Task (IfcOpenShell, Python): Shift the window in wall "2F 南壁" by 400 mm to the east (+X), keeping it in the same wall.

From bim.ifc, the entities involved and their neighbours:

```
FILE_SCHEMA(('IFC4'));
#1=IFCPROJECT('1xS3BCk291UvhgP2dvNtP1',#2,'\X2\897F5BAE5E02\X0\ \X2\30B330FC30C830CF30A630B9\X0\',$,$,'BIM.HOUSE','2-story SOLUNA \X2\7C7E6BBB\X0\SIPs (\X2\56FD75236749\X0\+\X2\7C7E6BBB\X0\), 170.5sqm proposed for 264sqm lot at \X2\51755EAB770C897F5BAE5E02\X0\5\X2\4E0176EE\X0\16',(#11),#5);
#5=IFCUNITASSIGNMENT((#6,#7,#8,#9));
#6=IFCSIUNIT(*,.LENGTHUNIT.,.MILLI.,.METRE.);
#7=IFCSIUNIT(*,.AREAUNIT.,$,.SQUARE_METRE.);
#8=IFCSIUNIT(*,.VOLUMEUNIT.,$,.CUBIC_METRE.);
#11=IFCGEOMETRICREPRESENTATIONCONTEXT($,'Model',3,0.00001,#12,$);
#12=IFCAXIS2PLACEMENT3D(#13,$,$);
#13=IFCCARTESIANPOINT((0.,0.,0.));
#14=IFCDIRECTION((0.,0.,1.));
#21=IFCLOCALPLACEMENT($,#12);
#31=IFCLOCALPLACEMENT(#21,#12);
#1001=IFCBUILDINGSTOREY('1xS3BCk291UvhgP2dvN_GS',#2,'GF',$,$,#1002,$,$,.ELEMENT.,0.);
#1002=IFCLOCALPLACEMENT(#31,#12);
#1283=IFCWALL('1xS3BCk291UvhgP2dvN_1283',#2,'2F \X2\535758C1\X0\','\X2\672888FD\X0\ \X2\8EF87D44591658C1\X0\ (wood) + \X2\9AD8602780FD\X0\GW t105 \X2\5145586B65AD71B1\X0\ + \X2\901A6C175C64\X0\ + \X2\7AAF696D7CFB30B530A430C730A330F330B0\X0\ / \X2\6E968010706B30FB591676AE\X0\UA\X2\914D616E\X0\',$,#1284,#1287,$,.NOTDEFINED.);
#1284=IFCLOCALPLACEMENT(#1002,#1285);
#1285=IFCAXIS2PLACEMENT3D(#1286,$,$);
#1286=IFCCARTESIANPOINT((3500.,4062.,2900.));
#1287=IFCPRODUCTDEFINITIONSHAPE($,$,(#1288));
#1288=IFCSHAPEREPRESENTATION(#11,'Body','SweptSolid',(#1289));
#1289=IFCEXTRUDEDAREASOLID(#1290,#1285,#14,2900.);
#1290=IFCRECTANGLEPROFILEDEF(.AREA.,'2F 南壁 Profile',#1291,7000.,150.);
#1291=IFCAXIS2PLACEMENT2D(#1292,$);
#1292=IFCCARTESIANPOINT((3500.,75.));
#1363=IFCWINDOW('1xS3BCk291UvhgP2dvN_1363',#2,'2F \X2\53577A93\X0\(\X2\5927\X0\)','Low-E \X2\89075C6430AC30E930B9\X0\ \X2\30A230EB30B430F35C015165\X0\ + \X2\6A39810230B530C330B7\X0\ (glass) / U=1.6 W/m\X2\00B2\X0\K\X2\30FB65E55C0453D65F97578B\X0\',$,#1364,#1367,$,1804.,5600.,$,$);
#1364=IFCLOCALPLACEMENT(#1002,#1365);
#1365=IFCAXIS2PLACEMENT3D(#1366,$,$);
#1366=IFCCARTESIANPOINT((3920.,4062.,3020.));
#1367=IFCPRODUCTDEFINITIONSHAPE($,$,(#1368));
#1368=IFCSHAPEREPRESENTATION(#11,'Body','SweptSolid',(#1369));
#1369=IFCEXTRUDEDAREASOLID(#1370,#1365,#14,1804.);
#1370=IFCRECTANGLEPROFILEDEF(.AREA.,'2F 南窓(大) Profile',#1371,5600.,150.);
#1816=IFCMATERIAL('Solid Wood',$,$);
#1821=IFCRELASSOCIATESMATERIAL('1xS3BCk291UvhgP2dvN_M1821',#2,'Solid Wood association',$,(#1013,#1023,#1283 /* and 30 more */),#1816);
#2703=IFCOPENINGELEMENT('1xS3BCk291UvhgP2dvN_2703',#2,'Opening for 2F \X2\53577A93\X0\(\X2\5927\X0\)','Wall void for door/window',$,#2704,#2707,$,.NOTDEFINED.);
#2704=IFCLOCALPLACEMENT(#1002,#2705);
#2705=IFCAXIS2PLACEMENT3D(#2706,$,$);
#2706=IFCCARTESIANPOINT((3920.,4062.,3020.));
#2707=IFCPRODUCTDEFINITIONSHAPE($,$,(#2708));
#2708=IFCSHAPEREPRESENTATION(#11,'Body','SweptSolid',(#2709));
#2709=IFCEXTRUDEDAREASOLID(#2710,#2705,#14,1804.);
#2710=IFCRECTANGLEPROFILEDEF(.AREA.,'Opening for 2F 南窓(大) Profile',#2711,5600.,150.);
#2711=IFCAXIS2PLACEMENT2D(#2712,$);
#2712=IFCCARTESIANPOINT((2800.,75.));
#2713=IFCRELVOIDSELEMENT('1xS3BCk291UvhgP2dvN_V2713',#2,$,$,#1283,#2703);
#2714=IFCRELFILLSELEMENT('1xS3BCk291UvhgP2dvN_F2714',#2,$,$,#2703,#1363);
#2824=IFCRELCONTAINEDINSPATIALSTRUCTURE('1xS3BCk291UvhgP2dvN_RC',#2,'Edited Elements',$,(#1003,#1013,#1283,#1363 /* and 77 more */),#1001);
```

```python
import ifcopenshell
import ifcopenshell.api.geometry
import ifcopenshell.util.placement
import ifcopenshell.util.unit

model = ifcopenshell.open("bim.ifc")
unit_scale = ifcopenshell.util.unit.calculate_unit_scale(model)

window = model.by_guid("1xS3BCk291UvhgP2dvN_1363")
opening = window.FillsVoids[0].RelatingOpeningElement
wall = opening.VoidsElements[0].RelatingBuildingElement

wall_matrix = ifcopenshell.util.placement.get_local_placement(wall.ObjectPlacement)
shift = wall_matrix[:3, 0] * 0.4 / unit_scale
before = ifcopenshell.util.placement.get_local_placement(window.ObjectPlacement)[:3, 3].copy()

# The window is not placed relative to its opening, so move both.
for product in (opening, window):
    matrix = ifcopenshell.util.placement.get_local_placement(product.ObjectPlacement)
    matrix[:3, 3] += shift
    ifcopenshell.api.geometry.edit_object_placement(model, product=product, matrix=matrix, is_si=False)

after = ifcopenshell.util.placement.get_local_placement(window.ObjectPlacement)[:3, 3]
print("window moved by", (after - before).round(3) + 0.0)

model.write("bim-out.ifc")
```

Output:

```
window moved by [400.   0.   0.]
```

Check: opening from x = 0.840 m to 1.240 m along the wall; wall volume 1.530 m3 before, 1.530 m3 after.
